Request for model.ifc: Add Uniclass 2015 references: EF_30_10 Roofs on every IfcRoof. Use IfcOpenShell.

First a look at what the model holds.

```python
import ifcopenshell

model = ifcopenshell.open("model.ifc")
print(model.schema)
print("classifications:", [c.Name for c in model.by_type("IfcClassification")])
for ifc_class in ("IfcDoor", "IfcRoof", "IfcStair", "IfcWall", "IfcWindow"):
    print(ifc_class, len(model.by_type(ifc_class)))
```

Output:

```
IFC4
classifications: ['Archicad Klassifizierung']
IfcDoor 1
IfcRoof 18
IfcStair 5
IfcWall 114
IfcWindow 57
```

```python
import ifcopenshell
import ifcopenshell.api.classification

model = ifcopenshell.open("model.ifc")

system = ifcopenshell.api.classification.add_classification(model, classification="Uniclass 2015")

codes = {
    "IfcRoof": ("EF_30_10", "Roofs"),
}
for ifc_class, (code, name) in codes.items():
    products = model.by_type(ifc_class)
    ifcopenshell.api.classification.add_reference(
        model, products=products, classification=system, identification=code, name=name
    )
    print(code, len(products))

model.write("model_v2.ifc")
```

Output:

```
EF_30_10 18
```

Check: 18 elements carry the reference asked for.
